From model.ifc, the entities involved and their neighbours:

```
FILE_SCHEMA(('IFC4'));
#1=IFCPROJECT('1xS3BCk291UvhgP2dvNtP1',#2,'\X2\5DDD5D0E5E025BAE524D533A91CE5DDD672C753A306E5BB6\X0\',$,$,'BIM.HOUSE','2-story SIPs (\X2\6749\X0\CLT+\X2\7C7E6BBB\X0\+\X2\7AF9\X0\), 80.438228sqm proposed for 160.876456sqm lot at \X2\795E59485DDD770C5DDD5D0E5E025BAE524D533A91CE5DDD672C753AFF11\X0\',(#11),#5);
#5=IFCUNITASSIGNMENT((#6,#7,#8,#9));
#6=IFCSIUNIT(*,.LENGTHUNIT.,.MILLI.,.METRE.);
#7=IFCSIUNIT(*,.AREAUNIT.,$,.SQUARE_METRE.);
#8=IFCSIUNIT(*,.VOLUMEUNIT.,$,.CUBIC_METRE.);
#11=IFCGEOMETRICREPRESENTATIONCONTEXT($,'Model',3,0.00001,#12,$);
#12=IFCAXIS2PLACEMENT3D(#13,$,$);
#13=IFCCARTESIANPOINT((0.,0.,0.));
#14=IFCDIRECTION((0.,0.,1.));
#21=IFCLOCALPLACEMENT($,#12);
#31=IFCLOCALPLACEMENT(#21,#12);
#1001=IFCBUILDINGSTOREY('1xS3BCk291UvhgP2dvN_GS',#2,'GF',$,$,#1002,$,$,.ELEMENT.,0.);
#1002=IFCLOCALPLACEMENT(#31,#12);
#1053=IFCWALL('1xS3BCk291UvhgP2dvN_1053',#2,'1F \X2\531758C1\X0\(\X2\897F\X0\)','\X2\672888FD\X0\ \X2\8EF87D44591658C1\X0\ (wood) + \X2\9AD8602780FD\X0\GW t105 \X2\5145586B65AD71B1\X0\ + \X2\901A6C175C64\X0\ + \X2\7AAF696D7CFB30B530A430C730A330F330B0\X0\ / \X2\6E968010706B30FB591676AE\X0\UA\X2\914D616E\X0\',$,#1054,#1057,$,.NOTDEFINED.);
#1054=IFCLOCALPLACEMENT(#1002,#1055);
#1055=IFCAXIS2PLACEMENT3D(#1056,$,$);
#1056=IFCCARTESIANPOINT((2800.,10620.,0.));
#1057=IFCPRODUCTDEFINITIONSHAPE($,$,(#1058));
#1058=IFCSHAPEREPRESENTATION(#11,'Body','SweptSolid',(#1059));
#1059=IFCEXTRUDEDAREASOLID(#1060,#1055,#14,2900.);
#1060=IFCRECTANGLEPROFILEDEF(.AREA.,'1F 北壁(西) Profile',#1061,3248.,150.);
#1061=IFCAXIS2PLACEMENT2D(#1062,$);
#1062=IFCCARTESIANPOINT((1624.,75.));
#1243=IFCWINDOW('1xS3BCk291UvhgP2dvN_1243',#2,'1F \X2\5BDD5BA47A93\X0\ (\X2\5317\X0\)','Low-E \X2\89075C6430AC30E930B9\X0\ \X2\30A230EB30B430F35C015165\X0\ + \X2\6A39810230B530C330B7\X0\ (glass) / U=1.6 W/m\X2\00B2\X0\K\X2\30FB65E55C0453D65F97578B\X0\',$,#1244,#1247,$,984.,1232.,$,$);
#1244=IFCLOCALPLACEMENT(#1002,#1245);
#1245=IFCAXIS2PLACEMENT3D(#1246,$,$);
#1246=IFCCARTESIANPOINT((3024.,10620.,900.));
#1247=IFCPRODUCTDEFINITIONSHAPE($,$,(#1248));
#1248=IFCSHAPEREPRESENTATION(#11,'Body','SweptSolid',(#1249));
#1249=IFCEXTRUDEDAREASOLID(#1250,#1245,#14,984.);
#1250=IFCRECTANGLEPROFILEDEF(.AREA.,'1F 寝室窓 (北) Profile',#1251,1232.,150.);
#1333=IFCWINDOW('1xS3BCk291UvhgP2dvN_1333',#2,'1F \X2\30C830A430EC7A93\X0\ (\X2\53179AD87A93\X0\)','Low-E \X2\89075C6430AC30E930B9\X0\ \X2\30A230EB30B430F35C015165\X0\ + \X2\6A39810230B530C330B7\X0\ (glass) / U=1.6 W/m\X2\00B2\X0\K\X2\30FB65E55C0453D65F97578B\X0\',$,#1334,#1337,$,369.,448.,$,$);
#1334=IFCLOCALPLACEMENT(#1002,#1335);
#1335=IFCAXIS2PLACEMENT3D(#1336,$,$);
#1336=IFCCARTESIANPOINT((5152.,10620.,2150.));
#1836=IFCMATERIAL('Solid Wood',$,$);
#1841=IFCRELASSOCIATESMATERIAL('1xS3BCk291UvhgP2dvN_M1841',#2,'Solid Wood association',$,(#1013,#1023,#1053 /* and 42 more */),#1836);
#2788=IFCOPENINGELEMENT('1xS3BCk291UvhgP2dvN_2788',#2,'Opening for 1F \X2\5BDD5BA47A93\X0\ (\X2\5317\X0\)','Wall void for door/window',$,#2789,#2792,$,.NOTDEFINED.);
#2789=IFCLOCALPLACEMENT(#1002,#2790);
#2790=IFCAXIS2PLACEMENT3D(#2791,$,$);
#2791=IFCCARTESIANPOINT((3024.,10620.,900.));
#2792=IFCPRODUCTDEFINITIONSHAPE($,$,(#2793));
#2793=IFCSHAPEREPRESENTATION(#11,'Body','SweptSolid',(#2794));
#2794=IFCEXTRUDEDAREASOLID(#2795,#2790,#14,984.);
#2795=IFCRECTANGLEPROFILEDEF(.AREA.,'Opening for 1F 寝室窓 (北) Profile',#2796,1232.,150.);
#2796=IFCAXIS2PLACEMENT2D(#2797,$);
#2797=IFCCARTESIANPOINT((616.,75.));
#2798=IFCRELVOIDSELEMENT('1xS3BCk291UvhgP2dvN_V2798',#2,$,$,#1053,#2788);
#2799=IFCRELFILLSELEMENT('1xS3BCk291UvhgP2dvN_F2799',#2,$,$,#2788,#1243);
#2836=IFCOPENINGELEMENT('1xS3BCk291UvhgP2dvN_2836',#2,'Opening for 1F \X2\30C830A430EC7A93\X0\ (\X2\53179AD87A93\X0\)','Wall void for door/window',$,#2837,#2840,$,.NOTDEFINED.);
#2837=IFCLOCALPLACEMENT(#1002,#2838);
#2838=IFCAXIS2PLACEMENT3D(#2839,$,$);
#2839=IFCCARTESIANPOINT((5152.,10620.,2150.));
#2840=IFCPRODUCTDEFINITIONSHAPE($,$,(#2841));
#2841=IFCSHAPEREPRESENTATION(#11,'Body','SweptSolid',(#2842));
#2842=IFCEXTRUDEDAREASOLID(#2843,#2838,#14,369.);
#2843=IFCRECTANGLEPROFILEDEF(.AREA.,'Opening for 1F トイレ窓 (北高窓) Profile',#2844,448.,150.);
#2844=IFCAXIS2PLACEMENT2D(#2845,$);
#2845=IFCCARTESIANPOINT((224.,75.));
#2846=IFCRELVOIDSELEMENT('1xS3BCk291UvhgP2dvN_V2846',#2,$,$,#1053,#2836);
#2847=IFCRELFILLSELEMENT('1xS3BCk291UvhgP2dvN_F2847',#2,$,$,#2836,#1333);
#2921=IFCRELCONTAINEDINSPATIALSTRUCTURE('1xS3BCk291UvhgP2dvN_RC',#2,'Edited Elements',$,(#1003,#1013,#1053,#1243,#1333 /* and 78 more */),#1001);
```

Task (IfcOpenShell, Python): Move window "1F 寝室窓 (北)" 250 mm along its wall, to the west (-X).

```python
import ifcopenshell
import ifcopenshell.api.geometry
import ifcopenshell.util.placement

model = ifcopenshell.open("model.ifc")

window = model.by_guid("1xS3BCk291UvhgP2dvN_1243")
opening = window.FillsVoids[0].RelatingOpeningElement
wall = opening.VoidsElements[0].RelatingBuildingElement

wall_matrix = ifcopenshell.util.placement.get_local_placement(wall.ObjectPlacement)
shift = wall_matrix[:3, 0] * -250.0
before = ifcopenshell.util.placement.get_local_placement(window.ObjectPlacement)[:3, 3].copy()

# The window is not placed relative to its opening, so move both.
for product in (opening, window):
    matrix = ifcopenshell.util.placement.get_local_placement(product.ObjectPlacement)
    matrix[:3, 3] += shift
    ifcopenshell.api.geometry.edit_object_placement(model, product=product, matrix=matrix, is_si=False)

after = ifcopenshell.util.placement.get_local_placement(window.ObjectPlacement)[:3, 3]
print("window moved by", (after - before).round(3) + 0.0)

model.write("model_updated.ifc")
```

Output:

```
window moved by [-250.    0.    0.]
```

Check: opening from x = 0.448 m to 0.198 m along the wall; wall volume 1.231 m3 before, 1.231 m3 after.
